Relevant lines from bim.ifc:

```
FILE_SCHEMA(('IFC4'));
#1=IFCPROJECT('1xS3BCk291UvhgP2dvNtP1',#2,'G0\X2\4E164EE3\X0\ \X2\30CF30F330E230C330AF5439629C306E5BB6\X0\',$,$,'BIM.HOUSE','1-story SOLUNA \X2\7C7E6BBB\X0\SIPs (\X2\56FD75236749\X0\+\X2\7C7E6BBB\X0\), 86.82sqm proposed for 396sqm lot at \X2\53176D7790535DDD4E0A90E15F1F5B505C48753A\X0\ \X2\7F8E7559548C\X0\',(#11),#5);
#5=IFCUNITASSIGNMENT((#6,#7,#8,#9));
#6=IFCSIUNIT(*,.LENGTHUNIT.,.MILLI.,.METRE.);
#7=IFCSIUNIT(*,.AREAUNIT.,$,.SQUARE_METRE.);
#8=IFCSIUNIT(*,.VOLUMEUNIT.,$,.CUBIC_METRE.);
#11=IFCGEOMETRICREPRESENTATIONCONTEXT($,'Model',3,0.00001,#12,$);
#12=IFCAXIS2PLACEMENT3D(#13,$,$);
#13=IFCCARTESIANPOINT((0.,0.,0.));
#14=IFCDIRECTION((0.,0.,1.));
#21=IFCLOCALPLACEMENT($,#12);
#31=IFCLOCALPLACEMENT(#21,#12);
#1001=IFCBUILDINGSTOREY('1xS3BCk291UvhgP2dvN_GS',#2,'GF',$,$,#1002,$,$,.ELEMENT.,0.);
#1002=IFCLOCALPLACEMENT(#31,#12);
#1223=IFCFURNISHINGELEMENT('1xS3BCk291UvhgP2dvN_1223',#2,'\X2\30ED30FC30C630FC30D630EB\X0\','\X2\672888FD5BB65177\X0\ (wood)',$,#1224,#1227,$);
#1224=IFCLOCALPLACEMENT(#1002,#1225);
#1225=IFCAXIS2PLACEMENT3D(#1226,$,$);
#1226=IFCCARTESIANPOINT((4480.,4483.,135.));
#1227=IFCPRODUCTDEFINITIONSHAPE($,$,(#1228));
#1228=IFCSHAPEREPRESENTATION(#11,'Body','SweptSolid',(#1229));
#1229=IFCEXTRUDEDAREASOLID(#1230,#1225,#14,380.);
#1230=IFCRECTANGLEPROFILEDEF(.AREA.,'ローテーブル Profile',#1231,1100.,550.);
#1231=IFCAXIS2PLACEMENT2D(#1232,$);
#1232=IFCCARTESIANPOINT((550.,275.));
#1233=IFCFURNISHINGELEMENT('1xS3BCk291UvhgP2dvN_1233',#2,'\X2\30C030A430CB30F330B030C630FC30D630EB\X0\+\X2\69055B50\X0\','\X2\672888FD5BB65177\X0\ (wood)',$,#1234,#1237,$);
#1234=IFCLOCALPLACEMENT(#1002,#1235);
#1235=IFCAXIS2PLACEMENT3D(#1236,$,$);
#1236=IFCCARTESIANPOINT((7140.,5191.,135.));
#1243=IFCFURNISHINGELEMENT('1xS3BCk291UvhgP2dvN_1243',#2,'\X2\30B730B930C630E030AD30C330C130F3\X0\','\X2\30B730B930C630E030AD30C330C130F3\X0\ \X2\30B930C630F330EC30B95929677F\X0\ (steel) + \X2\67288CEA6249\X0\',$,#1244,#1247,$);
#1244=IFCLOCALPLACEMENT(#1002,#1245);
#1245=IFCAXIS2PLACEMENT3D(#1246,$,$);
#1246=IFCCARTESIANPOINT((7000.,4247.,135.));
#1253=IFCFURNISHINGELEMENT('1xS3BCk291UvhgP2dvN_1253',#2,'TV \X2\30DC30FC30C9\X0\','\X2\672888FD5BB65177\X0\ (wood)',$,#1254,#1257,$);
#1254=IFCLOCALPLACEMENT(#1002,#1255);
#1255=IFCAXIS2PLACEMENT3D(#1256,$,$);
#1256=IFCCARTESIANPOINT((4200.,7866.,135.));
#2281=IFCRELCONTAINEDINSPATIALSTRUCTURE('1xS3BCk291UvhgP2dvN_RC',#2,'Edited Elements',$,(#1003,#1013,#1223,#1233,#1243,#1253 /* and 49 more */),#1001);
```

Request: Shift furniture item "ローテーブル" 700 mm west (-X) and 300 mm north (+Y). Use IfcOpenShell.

```python
import ifcopenshell
import ifcopenshell.api.geometry
import ifcopenshell.util.placement

model = ifcopenshell.open("bim.ifc")

item = model.by_guid("1xS3BCk291UvhgP2dvN_1223")
matrix = ifcopenshell.util.placement.get_local_placement(item.ObjectPlacement)
matrix[0, 3] -= 700.0
matrix[1, 3] += 300.0
ifcopenshell.api.geometry.edit_object_placement(model, product=item, matrix=matrix, is_si=False)

print(ifcopenshell.util.placement.get_local_placement(item.ObjectPlacement).round(3) + 0.0)

model.write("bim_edited.ifc")
```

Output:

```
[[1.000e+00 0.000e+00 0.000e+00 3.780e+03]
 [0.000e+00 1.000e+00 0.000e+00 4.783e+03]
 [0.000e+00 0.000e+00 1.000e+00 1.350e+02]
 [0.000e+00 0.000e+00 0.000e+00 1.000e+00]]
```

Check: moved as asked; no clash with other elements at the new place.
